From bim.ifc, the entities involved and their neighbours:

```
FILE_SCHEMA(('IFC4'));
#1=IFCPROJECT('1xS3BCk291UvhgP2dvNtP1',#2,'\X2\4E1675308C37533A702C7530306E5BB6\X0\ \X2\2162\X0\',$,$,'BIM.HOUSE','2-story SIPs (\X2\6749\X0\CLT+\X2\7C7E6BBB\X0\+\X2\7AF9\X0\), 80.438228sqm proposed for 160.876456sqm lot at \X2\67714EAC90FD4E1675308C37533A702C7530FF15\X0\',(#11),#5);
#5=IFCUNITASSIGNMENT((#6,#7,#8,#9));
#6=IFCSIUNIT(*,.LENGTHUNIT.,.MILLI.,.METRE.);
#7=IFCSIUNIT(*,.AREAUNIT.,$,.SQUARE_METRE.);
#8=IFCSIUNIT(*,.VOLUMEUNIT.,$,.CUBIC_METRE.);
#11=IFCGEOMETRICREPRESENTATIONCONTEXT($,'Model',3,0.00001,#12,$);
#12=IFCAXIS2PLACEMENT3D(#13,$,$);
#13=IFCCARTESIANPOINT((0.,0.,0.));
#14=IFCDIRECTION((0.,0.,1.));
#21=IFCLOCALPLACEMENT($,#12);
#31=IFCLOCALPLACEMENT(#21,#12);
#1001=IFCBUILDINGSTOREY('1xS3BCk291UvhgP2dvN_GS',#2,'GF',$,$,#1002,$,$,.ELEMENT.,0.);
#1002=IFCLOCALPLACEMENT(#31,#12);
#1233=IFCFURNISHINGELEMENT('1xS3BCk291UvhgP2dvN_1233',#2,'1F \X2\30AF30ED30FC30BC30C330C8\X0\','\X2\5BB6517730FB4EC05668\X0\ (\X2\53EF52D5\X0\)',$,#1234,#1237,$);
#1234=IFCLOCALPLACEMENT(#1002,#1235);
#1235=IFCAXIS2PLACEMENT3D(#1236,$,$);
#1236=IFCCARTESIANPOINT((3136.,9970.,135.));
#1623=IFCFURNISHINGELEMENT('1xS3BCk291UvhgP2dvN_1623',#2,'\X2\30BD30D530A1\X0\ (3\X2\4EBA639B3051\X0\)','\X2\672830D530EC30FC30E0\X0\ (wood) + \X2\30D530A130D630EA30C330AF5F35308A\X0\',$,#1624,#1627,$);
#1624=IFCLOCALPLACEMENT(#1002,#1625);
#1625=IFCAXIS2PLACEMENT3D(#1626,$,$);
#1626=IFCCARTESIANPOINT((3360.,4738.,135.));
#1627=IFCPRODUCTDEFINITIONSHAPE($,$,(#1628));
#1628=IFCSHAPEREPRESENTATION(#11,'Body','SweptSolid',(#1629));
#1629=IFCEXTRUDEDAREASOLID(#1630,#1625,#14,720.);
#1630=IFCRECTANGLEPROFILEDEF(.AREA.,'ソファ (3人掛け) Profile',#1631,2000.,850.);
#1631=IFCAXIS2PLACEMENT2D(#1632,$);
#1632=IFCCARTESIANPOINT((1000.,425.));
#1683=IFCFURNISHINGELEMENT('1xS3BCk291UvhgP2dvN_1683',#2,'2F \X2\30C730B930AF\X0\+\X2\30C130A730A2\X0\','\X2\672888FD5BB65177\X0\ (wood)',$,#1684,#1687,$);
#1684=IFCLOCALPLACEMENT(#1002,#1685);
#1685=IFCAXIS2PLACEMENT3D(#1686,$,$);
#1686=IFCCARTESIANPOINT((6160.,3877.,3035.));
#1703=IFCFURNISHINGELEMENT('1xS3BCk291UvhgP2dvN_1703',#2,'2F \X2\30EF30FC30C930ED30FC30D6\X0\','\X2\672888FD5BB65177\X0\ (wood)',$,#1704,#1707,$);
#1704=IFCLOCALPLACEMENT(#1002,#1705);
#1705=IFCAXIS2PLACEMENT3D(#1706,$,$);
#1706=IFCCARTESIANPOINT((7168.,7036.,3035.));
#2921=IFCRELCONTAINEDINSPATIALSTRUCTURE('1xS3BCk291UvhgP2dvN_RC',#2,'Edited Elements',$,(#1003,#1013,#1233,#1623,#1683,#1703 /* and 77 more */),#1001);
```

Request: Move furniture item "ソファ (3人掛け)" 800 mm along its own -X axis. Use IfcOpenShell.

```python
import ifcopenshell
import ifcopenshell.api.geometry
import ifcopenshell.util.placement
import ifcopenshell.util.unit

model = ifcopenshell.open("bim.ifc")
unit_scale = ifcopenshell.util.unit.calculate_unit_scale(model)

item = model.by_guid("1xS3BCk291UvhgP2dvN_1623")
matrix = ifcopenshell.util.placement.get_local_placement(item.ObjectPlacement)
matrix[:3, 3] -= matrix[:3, 0] * 0.8 / unit_scale
ifcopenshell.api.geometry.edit_object_placement(model, product=item, matrix=matrix, is_si=False)

print(ifcopenshell.util.placement.get_local_placement(item.ObjectPlacement).round(3) + 0.0)

model.write("bim_updated.ifc")
```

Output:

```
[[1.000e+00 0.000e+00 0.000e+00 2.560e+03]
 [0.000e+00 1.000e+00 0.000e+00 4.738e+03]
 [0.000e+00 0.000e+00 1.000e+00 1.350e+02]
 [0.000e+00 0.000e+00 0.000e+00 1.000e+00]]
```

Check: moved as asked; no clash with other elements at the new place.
